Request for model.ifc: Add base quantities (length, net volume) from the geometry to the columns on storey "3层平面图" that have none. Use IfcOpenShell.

First a look at what the model holds.

```python
import ifcopenshell
import ifcopenshell.util.element
import ifcopenshell.util.unit

model = ifcopenshell.open("model.ifc")
print(model.schema)
for unit_type in ("LENGTHUNIT", "AREAUNIT", "VOLUMEUNIT"):
    print(unit_type, ifcopenshell.util.unit.calculate_unit_scale(model, unit_type))
storey = next(s for s in model.by_type("IfcBuildingStorey") if s.Name == "3层平面图")
columns = [e for e in ifcopenshell.util.element.get_decomposition(storey) if e.is_a("IfcColumn")]
for e in sorted(columns, key=lambda e: e.id()):
    print(e.id(), e.is_a(), e.Name, list(ifcopenshell.util.element.get_psets(e, qtos_only=True)), sep=" | ")
```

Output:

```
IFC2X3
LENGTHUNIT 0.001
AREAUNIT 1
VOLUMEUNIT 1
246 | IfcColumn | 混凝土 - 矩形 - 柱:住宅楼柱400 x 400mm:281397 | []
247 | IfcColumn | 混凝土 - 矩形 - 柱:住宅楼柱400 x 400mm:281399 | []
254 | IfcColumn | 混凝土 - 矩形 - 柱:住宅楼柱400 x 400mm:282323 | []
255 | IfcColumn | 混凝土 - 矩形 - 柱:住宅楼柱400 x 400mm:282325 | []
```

```python
import ifcopenshell
import ifcopenshell.api.pset
import ifcopenshell.geom
import ifcopenshell.util.element
import ifcopenshell.util.shape
import ifcopenshell.util.unit

model = ifcopenshell.open("model.ifc")
unit_scale = ifcopenshell.util.unit.calculate_unit_scale(model)
volume_scale = ifcopenshell.util.unit.calculate_unit_scale(model, "VOLUMEUNIT")
settings = ifcopenshell.geom.settings()

storey = next(s for s in model.by_type("IfcBuildingStorey") if s.Name == "3层平面图")
columns = [e for e in ifcopenshell.util.element.get_decomposition(storey) if e.is_a("IfcColumn")]

for e in sorted(columns, key=lambda e: e.id()):
    if ifcopenshell.util.element.get_psets(e, qtos_only=True, should_inherit=False):
        continue
    # Geometry comes back in metres, in the element's own axes.
    shape = ifcopenshell.geom.create_shape(settings, e)
    values = {
        "Length": ifcopenshell.util.shape.get_z(shape.geometry) / unit_scale,
        "NetVolume": ifcopenshell.util.shape.get_volume(shape.geometry) / volume_scale,
    }
    qto = ifcopenshell.api.pset.add_qto(model, product=e, name="BaseQuantities")
    ifcopenshell.api.pset.edit_qto(model, qto=qto, properties=values)
    print(e.id(), {k: round(v, 3) for k, v in values.items()})

model.write("model-out.ifc")
```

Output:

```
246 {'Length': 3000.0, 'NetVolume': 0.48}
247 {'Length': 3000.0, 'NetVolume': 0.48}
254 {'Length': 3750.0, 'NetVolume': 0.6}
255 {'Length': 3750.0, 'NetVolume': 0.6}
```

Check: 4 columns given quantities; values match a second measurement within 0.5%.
